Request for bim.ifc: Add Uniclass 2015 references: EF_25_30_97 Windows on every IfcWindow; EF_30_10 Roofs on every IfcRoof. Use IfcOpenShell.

First a look at what the model holds.

```python
import ifcopenshell

model = ifcopenshell.open("bim.ifc")
print(model.schema)
print("classifications:", [c.Name for c in model.by_type("IfcClassification")])
for ifc_class in ("IfcDoor", "IfcRoof", "IfcStair", "IfcWall", "IfcWindow"):
    print(ifc_class, len(model.by_type(ifc_class)))
```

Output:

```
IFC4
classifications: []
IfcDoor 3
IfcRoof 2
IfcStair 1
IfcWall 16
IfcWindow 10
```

```python
import ifcopenshell
import ifcopenshell.api.classification

model = ifcopenshell.open("bim.ifc")

system = ifcopenshell.api.classification.add_classification(model, classification="Uniclass 2015")

codes = {
    "IfcWindow": ("EF_25_30_97", "Windows"),
    "IfcRoof": ("EF_30_10", "Roofs"),
}
for ifc_class, (code, name) in codes.items():
    products = model.by_type(ifc_class)
    ifcopenshell.api.classification.add_reference(
        model, products=products, classification=system, identification=code, name=name
    )
    print(code, len(products))

model.write("bim_edited.ifc")
```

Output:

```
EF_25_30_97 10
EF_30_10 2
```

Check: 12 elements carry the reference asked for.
